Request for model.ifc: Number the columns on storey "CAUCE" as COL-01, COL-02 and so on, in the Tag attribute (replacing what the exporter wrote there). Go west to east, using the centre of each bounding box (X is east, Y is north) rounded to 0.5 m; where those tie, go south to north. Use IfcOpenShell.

First a look at what the model holds.

```python
import ifcopenshell
import ifcopenshell.util.element
import ifcopenshell.util.placement

model = ifcopenshell.open("model.ifc")
print(model.schema)
storey = next(s for s in model.by_type("IfcBuildingStorey") if s.Name == "CAUCE")
columns = [e for e in ifcopenshell.util.element.get_decomposition(storey) if e.is_a("IfcColumn")]
for e in sorted(columns, key=lambda e: e.id()):
    origin = ifcopenshell.util.placement.get_local_placement(e.ObjectPlacement)[:3, 3]
    print(e.id(), e.Tag, e.Name, origin.round(2) + 0.0, sep=" | ")
```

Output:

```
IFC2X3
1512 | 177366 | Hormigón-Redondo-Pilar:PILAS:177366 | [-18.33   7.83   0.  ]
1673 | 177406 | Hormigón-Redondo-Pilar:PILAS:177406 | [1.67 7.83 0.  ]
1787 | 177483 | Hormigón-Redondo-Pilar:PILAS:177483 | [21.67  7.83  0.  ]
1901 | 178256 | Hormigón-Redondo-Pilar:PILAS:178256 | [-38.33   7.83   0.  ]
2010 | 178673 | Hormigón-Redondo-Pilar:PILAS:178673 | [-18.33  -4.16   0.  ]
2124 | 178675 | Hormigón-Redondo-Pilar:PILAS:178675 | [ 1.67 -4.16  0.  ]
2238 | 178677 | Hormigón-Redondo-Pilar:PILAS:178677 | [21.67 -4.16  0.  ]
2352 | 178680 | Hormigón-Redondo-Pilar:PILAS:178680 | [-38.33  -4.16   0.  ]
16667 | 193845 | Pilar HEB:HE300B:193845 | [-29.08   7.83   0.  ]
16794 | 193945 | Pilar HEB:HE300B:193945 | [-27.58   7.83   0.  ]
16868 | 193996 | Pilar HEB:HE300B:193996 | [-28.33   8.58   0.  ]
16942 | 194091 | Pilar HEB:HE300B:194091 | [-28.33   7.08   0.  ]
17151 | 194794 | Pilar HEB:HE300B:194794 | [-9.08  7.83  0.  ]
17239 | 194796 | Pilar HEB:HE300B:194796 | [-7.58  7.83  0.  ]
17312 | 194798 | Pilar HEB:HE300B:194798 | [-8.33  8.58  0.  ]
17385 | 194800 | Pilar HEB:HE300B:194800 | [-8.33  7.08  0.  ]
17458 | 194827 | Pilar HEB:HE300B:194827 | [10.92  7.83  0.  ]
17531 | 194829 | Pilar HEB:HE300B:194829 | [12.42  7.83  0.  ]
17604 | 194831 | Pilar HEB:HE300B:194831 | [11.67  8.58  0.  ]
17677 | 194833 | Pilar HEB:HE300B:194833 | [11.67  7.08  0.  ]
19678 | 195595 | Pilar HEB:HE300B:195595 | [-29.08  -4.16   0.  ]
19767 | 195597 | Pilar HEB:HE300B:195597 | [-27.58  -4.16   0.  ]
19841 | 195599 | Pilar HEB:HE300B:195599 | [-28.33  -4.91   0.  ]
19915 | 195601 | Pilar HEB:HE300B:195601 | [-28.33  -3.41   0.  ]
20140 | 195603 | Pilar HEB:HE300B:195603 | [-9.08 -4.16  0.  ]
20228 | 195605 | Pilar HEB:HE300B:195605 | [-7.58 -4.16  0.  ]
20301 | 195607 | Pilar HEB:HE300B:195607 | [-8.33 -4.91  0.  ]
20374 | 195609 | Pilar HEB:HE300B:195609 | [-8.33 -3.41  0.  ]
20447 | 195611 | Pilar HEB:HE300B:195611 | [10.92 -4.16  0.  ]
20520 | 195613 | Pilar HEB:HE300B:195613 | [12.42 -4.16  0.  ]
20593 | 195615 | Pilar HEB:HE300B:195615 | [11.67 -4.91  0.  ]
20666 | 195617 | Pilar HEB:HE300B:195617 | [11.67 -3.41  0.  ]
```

```python
import ifcopenshell
import ifcopenshell.geom
import ifcopenshell.util.element
import ifcopenshell.util.shape

model = ifcopenshell.open("model.ifc")
settings = ifcopenshell.geom.settings()
settings.set("use-world-coords", True)


def centre(element):
    shape = ifcopenshell.geom.create_shape(settings, element)
    return ifcopenshell.util.shape.get_bbox_centroid(shape.geometry)


storey = next(s for s in model.by_type("IfcBuildingStorey") if s.Name == "CAUCE")
columns = [e for e in ifcopenshell.util.element.get_decomposition(storey) if e.is_a("IfcColumn")]

# Insertion points can sit at a corner or the storey origin, so sort by the geometry (in metres).
centres = {e: centre(e) for e in columns}
columns.sort(key=lambda e: (round(centres[e][0] / 0.5), centres[e][1]))

for i, e in enumerate(columns, start=1):
    number = f"COL-{i:02d}"
    e.Tag = number
    print(e.id(), number)

model.write("model-out.ifc")
```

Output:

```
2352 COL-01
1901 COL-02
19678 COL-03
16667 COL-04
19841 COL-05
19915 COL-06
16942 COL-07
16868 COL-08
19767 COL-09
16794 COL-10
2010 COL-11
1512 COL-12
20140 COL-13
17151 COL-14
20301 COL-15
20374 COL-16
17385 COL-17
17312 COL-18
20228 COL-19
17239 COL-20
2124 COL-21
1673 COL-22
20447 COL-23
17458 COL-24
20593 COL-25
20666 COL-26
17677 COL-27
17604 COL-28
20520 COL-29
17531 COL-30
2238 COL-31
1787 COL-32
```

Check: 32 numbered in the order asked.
